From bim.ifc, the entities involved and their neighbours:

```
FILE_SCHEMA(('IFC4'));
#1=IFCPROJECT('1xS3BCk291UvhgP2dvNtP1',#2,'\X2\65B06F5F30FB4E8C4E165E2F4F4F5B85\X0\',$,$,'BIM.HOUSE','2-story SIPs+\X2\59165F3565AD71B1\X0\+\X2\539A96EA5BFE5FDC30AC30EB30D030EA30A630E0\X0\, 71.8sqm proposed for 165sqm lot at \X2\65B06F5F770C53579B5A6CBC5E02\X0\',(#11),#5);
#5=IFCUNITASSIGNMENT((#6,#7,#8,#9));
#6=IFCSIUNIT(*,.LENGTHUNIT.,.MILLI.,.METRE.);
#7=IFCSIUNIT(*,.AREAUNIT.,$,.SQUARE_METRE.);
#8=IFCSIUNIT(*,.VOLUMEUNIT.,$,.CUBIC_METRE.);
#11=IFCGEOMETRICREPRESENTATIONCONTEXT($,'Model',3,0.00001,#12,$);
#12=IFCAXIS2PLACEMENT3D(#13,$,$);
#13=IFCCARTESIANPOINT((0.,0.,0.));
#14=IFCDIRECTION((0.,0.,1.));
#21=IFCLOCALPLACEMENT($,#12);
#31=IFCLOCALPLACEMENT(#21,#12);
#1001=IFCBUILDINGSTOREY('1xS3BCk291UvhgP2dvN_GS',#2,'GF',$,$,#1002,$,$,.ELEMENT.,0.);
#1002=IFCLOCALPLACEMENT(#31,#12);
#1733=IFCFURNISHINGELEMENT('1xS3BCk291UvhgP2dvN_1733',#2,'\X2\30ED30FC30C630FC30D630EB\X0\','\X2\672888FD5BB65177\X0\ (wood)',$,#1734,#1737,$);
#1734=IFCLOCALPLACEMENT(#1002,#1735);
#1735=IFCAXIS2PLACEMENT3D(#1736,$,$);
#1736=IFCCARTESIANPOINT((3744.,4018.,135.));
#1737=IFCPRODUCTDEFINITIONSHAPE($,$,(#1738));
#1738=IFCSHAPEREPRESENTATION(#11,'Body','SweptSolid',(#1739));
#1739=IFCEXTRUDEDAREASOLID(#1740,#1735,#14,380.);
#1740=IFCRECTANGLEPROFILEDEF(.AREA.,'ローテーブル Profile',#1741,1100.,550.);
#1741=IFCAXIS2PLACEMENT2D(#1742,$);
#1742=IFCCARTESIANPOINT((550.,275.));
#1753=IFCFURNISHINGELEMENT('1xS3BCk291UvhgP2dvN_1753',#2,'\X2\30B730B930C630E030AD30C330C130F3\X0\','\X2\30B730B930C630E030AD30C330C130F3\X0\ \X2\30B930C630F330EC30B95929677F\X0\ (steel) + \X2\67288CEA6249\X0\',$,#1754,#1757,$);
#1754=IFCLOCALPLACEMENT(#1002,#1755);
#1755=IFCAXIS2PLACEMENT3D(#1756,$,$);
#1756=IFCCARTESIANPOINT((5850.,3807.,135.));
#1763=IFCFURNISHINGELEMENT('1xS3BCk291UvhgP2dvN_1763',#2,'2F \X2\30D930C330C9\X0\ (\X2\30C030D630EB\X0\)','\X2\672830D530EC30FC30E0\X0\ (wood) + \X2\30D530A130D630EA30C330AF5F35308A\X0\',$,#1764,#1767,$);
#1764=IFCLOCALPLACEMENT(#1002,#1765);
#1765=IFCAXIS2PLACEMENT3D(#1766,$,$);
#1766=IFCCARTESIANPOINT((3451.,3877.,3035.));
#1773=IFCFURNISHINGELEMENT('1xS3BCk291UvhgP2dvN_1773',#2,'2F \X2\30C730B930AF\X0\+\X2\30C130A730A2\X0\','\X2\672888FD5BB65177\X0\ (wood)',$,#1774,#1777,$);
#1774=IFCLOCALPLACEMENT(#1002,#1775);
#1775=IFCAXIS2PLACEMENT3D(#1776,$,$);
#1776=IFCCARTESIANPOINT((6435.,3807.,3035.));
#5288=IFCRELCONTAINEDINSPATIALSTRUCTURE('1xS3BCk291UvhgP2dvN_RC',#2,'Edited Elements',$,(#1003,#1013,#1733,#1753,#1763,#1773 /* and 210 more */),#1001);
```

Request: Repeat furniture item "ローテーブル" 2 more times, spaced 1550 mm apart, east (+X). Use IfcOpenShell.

```python
import numpy as np
import ifcopenshell
import ifcopenshell.api.geometry
import ifcopenshell.api.root
import ifcopenshell.util.element
import ifcopenshell.util.placement
import ifcopenshell.util.unit

model = ifcopenshell.open("bim.ifc")
unit_scale = ifcopenshell.util.unit.calculate_unit_scale(model)


def reuse_history(source, copy):
    """copy_class also copies each property set's owner history, people and application; keep the originals."""
    for rel in copy.IsDefinedBy:
        if rel.is_a("IfcRelDefinesByProperties") and (history := rel.RelatingPropertyDefinition.OwnerHistory):
            rel.RelatingPropertyDefinition.OwnerHistory = source.OwnerHistory
            ifcopenshell.util.element.remove_deep2(model, history)


source = model.by_guid("1xS3BCk291UvhgP2dvN_1733")
base = ifcopenshell.util.placement.get_local_placement(source.ObjectPlacement)
step = np.array([1.0, 0.0, 0.0]) * 1.55 / unit_scale

for i in range(1, 3):
    copy = ifcopenshell.api.root.copy_class(model, product=source)
    copy.Representation = ifcopenshell.util.element.copy_deep(
        model, source.Representation, exclude=["IfcGeometricRepresentationContext", "IfcRepresentationMap"]
    )
    reuse_history(source, copy)
    matrix = base.copy()
    matrix[:3, 3] += i * step
    print("added at", matrix[:3, 3].round(3) + 0.0)
    ifcopenshell.api.geometry.edit_object_placement(model, product=copy, matrix=matrix, is_si=False)

model.write("bim_rev.ifc")
```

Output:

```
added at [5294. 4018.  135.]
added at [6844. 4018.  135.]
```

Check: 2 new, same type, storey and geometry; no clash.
